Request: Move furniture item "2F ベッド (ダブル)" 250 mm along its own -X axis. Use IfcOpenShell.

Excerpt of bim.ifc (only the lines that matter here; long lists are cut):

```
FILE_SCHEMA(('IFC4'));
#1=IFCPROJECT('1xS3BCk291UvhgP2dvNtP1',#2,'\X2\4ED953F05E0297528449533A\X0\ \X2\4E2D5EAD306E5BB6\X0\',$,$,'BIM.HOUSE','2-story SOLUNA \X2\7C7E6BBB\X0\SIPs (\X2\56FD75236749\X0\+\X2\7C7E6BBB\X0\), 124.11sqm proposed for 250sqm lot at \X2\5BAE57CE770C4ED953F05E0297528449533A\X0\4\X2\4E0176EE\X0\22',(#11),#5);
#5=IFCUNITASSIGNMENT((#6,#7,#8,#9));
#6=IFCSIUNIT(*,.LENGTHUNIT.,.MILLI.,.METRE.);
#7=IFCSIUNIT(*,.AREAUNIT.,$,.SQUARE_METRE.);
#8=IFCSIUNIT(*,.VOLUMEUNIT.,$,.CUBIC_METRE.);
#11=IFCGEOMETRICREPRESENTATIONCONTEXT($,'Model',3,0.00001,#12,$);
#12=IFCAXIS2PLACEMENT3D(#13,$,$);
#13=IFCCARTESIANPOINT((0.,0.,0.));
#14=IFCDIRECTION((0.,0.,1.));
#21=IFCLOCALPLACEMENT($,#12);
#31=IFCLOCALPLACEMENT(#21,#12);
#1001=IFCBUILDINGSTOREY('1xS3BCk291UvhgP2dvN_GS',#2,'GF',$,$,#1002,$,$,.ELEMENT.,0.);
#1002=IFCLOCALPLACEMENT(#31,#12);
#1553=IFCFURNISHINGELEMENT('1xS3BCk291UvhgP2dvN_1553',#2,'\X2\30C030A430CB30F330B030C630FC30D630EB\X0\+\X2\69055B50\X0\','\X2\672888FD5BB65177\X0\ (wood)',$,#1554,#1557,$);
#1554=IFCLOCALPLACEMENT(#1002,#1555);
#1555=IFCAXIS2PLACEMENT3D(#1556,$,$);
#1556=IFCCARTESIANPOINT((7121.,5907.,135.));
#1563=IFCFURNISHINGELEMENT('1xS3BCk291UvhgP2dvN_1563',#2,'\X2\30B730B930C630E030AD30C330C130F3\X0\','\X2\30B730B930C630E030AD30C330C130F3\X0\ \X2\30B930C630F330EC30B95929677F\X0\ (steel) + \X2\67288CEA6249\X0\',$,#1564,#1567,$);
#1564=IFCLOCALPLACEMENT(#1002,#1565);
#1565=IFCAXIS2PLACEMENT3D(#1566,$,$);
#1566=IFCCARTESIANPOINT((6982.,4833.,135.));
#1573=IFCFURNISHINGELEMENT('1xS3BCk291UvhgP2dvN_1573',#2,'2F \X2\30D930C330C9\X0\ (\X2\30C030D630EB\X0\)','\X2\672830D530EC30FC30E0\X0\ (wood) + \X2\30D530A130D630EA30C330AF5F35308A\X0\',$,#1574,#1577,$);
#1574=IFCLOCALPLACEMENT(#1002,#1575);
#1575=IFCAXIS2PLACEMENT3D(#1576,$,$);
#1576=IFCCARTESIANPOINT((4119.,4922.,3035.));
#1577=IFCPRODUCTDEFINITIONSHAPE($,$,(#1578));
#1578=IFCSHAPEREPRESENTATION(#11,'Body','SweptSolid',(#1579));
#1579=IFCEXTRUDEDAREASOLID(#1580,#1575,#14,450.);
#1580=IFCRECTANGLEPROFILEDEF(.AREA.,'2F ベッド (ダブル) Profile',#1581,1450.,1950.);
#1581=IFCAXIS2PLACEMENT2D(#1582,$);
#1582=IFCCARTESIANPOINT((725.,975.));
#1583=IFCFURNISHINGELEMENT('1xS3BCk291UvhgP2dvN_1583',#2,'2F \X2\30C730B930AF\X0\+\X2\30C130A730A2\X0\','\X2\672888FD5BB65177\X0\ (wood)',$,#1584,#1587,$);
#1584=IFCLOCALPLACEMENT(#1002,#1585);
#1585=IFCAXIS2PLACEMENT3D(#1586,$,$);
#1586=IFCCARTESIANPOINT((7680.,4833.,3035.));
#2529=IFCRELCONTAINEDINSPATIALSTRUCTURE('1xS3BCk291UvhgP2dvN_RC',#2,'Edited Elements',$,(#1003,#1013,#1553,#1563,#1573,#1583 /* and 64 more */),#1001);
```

```python
import ifcopenshell
import ifcopenshell.api.geometry
import ifcopenshell.util.placement

model = ifcopenshell.open("bim.ifc")

item = model.by_guid("1xS3BCk291UvhgP2dvN_1573")
matrix = ifcopenshell.util.placement.get_local_placement(item.ObjectPlacement)
matrix[:3, 3] -= matrix[:3, 0] * 250.0
ifcopenshell.api.geometry.edit_object_placement(model, product=item, matrix=matrix, is_si=False)

print(ifcopenshell.util.placement.get_local_placement(item.ObjectPlacement).round(3) + 0.0)

model.write("bim_rev.ifc")
```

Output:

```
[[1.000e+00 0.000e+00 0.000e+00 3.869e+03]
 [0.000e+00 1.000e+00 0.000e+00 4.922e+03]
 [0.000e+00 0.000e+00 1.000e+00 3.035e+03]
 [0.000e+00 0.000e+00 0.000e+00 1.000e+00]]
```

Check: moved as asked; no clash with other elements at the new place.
